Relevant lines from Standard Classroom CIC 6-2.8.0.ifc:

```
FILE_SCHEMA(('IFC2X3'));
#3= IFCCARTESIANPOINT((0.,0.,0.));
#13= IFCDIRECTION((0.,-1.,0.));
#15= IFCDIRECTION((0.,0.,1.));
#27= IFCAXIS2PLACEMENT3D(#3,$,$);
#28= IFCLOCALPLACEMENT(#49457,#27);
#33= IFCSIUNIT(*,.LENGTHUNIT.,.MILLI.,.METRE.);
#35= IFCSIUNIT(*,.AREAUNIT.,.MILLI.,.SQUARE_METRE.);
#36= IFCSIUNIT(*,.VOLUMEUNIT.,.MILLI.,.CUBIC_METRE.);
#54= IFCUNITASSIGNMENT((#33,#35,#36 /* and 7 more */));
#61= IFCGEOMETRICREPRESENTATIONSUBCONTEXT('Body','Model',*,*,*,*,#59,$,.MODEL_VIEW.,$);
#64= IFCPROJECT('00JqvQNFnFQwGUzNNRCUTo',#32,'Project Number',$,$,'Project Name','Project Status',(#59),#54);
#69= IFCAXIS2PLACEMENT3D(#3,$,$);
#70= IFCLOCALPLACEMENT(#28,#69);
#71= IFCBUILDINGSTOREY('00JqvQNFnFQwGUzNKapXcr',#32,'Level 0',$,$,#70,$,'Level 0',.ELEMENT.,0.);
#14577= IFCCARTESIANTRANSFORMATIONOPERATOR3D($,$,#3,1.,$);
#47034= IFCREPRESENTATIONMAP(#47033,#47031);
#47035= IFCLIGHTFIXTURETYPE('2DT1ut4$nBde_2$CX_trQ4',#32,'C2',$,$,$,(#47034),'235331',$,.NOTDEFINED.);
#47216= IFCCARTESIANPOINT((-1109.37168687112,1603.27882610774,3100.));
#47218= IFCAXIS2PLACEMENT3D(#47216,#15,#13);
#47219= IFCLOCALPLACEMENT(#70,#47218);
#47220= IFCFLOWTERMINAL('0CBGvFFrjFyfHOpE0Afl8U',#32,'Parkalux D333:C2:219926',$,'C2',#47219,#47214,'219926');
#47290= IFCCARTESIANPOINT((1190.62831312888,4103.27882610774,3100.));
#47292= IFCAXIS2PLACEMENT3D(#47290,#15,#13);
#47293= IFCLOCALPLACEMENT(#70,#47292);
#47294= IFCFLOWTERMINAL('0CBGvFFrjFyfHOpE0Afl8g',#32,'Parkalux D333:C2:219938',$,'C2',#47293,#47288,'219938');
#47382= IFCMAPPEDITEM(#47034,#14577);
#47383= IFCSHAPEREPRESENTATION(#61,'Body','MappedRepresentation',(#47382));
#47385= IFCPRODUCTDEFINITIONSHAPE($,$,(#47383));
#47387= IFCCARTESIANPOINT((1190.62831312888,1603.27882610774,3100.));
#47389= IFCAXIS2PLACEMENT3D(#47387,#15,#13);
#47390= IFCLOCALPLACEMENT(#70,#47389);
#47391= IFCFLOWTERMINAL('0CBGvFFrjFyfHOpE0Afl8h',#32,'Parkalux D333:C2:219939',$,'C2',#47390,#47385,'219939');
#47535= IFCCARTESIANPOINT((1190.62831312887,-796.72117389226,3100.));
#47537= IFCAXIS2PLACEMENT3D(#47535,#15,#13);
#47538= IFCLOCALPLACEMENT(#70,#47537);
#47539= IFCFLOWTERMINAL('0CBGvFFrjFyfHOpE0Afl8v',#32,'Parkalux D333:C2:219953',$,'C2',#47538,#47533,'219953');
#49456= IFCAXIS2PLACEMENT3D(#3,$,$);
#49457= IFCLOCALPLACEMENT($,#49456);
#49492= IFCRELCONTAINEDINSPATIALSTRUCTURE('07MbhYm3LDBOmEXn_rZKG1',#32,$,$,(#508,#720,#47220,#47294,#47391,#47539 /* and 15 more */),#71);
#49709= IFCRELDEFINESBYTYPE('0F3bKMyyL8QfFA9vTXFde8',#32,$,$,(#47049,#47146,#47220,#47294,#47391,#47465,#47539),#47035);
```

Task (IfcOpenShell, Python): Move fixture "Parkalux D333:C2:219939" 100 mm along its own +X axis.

```python
import ifcopenshell
import ifcopenshell.api.geometry
import ifcopenshell.util.placement
import ifcopenshell.util.unit

model = ifcopenshell.open("Standard Classroom CIC 6-2.8.0.ifc")
unit_scale = ifcopenshell.util.unit.calculate_unit_scale(model)

item = model.by_guid("0CBGvFFrjFyfHOpE0Afl8h")
matrix = ifcopenshell.util.placement.get_local_placement(item.ObjectPlacement)
matrix[:3, 3] += matrix[:3, 0] * 0.1 / unit_scale
ifcopenshell.api.geometry.edit_object_placement(model, product=item, matrix=matrix, is_si=False)

print(ifcopenshell.util.placement.get_local_placement(item.ObjectPlacement).round(3) + 0.0)

model.write("Standard Classroom CIC 6-2.8.0_updated.ifc")
```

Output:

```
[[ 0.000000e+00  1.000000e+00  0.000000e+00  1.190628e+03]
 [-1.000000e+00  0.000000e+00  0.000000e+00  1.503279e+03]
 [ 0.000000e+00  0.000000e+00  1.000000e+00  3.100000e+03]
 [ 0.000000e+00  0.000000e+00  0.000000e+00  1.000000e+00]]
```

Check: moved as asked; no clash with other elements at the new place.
